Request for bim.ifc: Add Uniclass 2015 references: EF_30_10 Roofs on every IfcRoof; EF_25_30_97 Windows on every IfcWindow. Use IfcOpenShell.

First a look at what the model holds.

```python
import ifcopenshell

model = ifcopenshell.open("bim.ifc")
print(model.schema)
print("classifications:", [c.Name for c in model.by_type("IfcClassification")])
for ifc_class in ("IfcDoor", "IfcRoof", "IfcStair", "IfcWall", "IfcWindow"):
    print(ifc_class, len(model.by_type(ifc_class)))
```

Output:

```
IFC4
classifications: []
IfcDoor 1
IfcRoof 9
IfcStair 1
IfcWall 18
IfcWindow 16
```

```python
import ifcopenshell
import ifcopenshell.api.classification

model = ifcopenshell.open("bim.ifc")

system = ifcopenshell.api.classification.add_classification(model, classification="Uniclass 2015")

codes = {
    "IfcRoof": ("EF_30_10", "Roofs"),
    "IfcWindow": ("EF_25_30_97", "Windows"),
}
for ifc_class, (code, name) in codes.items():
    products = model.by_type(ifc_class)
    ifcopenshell.api.classification.add_reference(
        model, products=products, classification=system, identification=code, name=name
    )
    print(code, len(products))

model.write("bim_rev.ifc")
```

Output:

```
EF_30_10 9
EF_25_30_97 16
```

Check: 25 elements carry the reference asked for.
